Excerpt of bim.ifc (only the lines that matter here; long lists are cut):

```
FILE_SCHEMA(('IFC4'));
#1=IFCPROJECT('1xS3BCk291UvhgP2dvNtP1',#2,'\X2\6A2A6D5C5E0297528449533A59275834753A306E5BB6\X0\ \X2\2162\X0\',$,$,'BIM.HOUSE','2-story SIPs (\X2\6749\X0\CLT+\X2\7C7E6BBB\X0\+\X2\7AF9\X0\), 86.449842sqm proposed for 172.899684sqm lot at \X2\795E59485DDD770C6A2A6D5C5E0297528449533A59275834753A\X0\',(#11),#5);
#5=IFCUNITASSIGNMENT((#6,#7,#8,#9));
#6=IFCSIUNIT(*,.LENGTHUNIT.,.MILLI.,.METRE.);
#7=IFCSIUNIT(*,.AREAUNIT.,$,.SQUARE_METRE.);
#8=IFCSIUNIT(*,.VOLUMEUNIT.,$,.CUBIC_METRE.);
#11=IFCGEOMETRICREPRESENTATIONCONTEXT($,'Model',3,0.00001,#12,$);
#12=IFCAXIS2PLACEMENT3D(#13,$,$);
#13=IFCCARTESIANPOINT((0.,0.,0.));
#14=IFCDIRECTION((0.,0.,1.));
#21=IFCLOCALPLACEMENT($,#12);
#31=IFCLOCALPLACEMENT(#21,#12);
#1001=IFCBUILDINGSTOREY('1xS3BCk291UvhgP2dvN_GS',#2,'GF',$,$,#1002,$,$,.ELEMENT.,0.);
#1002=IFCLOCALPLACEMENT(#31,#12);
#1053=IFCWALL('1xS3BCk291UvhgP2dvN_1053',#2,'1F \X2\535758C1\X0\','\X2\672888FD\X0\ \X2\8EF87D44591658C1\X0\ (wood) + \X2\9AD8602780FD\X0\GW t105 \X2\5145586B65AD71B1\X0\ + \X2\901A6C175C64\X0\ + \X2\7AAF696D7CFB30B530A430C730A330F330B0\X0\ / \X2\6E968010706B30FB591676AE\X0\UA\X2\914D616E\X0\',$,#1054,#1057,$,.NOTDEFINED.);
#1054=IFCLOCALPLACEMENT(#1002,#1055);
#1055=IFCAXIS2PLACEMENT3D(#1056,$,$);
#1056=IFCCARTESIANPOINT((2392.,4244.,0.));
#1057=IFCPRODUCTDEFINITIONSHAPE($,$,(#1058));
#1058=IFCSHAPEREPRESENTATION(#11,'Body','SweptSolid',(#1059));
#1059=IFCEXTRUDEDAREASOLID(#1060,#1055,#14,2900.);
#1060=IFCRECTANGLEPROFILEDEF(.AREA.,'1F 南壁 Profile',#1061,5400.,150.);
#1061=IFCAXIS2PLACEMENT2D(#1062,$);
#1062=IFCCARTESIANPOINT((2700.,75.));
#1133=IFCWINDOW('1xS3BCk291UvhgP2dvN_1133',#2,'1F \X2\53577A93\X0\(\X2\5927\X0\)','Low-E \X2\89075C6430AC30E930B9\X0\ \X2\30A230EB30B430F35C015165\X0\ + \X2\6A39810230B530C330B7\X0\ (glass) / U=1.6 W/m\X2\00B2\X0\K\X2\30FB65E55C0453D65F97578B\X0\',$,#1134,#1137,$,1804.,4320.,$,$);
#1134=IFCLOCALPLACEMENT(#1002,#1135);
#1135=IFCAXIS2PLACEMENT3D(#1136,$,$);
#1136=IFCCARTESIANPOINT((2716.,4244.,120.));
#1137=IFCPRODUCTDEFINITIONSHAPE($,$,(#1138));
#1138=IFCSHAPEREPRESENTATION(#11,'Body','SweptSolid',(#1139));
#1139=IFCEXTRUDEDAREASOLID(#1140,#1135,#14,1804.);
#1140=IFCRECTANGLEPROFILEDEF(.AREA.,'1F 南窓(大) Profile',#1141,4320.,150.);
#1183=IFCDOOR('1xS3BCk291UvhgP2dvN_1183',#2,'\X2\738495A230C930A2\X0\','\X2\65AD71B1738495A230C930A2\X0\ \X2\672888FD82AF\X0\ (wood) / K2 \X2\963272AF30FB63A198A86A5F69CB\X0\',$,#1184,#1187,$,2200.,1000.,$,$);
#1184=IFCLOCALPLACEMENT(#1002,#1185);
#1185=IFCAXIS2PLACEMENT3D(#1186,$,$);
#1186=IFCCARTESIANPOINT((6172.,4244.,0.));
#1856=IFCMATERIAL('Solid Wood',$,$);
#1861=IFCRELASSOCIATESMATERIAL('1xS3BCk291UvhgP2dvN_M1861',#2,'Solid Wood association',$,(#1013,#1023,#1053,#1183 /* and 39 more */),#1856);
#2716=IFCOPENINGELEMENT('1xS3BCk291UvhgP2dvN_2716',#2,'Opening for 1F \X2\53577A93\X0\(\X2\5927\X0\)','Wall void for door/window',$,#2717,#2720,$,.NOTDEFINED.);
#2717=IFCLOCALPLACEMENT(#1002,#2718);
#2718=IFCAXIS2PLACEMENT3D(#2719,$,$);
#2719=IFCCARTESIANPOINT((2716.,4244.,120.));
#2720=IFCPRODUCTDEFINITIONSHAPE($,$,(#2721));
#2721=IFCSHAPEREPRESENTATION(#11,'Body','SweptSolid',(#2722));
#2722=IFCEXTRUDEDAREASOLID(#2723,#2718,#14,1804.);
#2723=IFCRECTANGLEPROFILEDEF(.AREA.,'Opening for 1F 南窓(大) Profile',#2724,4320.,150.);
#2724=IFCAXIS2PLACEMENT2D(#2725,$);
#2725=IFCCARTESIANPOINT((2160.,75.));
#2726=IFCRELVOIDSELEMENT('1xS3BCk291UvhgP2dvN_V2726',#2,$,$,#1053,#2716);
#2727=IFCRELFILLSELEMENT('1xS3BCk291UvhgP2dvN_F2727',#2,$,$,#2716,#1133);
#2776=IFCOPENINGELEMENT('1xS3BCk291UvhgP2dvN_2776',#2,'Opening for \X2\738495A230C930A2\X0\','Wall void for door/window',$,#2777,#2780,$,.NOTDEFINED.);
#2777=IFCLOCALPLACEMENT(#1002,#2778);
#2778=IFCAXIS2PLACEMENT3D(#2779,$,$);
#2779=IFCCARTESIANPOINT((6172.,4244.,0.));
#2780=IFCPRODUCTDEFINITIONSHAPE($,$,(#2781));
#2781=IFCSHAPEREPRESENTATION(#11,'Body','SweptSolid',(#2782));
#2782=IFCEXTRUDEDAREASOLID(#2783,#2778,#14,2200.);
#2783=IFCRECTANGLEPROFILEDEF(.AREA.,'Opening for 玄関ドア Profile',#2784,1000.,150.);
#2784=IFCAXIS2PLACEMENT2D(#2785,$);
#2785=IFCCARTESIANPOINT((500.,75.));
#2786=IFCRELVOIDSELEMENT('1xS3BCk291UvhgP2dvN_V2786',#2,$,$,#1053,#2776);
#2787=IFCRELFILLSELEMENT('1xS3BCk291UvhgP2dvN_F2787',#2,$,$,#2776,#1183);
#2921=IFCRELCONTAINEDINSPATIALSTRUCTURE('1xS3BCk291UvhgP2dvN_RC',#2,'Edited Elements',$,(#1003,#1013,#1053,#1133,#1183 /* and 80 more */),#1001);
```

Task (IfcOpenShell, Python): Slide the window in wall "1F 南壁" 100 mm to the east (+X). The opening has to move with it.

```python
import ifcopenshell
import ifcopenshell.api.geometry
import ifcopenshell.util.placement
import ifcopenshell.util.unit

model = ifcopenshell.open("bim.ifc")
unit_scale = ifcopenshell.util.unit.calculate_unit_scale(model)

window = model.by_id(1133)
opening = window.FillsVoids[0].RelatingOpeningElement
wall = opening.VoidsElements[0].RelatingBuildingElement

wall_matrix = ifcopenshell.util.placement.get_local_placement(wall.ObjectPlacement)
shift = wall_matrix[:3, 0] * 0.1 / unit_scale
before = ifcopenshell.util.placement.get_local_placement(window.ObjectPlacement)[:3, 3].copy()

# The window is not placed relative to its opening, so move both.
for product in (opening, window):
    matrix = ifcopenshell.util.placement.get_local_placement(product.ObjectPlacement)
    matrix[:3, 3] += shift
    ifcopenshell.api.geometry.edit_object_placement(model, product=product, matrix=matrix, is_si=False)

after = ifcopenshell.util.placement.get_local_placement(window.ObjectPlacement)[:3, 3]
print("window moved by", (after - before).round(3) + 0.0)

model.write("bim-out.ifc")
```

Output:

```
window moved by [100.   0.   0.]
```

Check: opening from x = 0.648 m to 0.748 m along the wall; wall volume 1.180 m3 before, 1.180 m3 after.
